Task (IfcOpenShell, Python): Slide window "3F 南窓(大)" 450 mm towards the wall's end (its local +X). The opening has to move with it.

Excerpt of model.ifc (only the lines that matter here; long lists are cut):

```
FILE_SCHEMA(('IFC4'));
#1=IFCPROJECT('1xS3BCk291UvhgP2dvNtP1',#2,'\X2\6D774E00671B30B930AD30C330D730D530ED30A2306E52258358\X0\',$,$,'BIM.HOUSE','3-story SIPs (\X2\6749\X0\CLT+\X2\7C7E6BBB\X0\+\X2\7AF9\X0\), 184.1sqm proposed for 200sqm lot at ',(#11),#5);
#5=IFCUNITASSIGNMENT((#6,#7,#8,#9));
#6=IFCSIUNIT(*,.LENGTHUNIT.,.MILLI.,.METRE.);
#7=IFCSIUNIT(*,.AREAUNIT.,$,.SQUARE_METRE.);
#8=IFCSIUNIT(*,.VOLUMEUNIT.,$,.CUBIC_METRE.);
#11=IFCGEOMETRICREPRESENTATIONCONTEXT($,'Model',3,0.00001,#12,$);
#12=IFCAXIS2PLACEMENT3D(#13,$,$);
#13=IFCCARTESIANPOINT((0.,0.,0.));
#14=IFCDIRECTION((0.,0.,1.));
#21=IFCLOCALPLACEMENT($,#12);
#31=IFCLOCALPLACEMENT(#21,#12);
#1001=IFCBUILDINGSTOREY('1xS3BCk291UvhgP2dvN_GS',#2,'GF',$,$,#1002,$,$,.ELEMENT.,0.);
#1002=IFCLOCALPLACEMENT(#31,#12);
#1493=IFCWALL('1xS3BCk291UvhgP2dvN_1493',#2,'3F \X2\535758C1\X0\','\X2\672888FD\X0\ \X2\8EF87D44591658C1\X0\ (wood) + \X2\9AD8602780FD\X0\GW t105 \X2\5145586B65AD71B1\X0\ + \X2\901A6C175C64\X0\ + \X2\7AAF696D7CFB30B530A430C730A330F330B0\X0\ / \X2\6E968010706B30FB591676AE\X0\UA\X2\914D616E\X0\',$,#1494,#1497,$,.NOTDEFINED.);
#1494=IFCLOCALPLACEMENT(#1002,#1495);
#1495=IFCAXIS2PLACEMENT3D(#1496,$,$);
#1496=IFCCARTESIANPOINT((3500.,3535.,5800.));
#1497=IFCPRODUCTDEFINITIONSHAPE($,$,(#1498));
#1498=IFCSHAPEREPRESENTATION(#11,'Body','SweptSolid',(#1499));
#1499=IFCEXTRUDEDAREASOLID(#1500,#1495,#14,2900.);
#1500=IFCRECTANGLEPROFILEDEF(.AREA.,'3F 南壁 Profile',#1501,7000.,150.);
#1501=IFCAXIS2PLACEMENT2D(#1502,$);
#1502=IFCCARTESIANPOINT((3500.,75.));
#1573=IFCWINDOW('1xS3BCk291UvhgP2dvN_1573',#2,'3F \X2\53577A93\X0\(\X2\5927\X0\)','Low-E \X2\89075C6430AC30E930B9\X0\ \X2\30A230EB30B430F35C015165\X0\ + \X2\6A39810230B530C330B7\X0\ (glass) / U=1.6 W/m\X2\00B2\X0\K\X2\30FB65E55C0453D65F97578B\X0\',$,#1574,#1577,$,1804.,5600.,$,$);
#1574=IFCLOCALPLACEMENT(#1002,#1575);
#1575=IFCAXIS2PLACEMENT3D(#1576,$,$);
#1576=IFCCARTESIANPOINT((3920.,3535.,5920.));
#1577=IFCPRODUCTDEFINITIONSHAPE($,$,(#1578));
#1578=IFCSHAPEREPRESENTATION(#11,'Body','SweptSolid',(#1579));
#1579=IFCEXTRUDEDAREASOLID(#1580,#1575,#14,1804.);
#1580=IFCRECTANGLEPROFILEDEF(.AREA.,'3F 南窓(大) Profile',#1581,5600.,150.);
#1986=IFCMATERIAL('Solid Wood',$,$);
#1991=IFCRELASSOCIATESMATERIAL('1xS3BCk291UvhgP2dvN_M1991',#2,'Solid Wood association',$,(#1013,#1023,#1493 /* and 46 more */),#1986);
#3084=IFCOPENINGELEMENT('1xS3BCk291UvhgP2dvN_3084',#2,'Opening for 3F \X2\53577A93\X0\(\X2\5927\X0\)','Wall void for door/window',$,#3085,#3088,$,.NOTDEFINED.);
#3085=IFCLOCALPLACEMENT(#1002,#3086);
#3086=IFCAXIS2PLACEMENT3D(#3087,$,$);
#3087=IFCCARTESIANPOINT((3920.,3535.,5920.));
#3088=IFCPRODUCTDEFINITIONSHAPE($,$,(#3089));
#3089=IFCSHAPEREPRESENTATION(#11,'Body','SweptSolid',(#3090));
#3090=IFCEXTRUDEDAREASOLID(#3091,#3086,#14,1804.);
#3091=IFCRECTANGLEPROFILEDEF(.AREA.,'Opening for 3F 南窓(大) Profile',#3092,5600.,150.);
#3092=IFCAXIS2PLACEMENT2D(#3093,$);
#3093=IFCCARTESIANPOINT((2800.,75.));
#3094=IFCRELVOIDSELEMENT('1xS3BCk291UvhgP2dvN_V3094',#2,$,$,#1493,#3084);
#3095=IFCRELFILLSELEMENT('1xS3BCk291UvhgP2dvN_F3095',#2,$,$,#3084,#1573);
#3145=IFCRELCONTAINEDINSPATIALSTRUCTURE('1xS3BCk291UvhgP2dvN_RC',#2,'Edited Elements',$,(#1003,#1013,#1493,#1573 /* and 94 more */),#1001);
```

```python
import ifcopenshell
import ifcopenshell.api.geometry
import ifcopenshell.util.placement
import ifcopenshell.util.unit

model = ifcopenshell.open("model.ifc")
unit_scale = ifcopenshell.util.unit.calculate_unit_scale(model)

window = model.by_guid("1xS3BCk291UvhgP2dvN_1573")
opening = window.FillsVoids[0].RelatingOpeningElement
wall = opening.VoidsElements[0].RelatingBuildingElement

wall_matrix = ifcopenshell.util.placement.get_local_placement(wall.ObjectPlacement)
shift = wall_matrix[:3, 0] * 0.45 / unit_scale
before = ifcopenshell.util.placement.get_local_placement(window.ObjectPlacement)[:3, 3].copy()

# The window is not placed relative to its opening, so move both.
for product in (opening, window):
    matrix = ifcopenshell.util.placement.get_local_placement(product.ObjectPlacement)
    matrix[:3, 3] += shift
    ifcopenshell.api.geometry.edit_object_placement(model, product=product, matrix=matrix, is_si=False)

after = ifcopenshell.util.placement.get_local_placement(window.ObjectPlacement)[:3, 3]
print("window moved by", (after - before).round(3) + 0.0)

model.write("model_v2.ifc")
```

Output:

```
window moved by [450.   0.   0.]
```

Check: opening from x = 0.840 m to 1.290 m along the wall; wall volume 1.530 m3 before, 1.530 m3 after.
